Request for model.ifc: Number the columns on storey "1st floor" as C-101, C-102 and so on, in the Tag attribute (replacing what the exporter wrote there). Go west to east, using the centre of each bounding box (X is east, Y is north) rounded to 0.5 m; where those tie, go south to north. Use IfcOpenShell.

First a look at what the model holds.

```python
import ifcopenshell
import ifcopenshell.util.element
import ifcopenshell.util.placement

model = ifcopenshell.open("model.ifc")
print(model.schema)
storey = next(s for s in model.by_type("IfcBuildingStorey") if s.Name == "1st floor")
columns = [e for e in ifcopenshell.util.element.get_decomposition(storey) if e.is_a("IfcColumn")]
for e in sorted(columns, key=lambda e: e.id()):
    origin = ifcopenshell.util.placement.get_local_placement(e.ObjectPlacement)[:3, 3]
    print(e.id(), e.Tag, e.Name, origin.round(2) + 0.0, sep=" | ")
```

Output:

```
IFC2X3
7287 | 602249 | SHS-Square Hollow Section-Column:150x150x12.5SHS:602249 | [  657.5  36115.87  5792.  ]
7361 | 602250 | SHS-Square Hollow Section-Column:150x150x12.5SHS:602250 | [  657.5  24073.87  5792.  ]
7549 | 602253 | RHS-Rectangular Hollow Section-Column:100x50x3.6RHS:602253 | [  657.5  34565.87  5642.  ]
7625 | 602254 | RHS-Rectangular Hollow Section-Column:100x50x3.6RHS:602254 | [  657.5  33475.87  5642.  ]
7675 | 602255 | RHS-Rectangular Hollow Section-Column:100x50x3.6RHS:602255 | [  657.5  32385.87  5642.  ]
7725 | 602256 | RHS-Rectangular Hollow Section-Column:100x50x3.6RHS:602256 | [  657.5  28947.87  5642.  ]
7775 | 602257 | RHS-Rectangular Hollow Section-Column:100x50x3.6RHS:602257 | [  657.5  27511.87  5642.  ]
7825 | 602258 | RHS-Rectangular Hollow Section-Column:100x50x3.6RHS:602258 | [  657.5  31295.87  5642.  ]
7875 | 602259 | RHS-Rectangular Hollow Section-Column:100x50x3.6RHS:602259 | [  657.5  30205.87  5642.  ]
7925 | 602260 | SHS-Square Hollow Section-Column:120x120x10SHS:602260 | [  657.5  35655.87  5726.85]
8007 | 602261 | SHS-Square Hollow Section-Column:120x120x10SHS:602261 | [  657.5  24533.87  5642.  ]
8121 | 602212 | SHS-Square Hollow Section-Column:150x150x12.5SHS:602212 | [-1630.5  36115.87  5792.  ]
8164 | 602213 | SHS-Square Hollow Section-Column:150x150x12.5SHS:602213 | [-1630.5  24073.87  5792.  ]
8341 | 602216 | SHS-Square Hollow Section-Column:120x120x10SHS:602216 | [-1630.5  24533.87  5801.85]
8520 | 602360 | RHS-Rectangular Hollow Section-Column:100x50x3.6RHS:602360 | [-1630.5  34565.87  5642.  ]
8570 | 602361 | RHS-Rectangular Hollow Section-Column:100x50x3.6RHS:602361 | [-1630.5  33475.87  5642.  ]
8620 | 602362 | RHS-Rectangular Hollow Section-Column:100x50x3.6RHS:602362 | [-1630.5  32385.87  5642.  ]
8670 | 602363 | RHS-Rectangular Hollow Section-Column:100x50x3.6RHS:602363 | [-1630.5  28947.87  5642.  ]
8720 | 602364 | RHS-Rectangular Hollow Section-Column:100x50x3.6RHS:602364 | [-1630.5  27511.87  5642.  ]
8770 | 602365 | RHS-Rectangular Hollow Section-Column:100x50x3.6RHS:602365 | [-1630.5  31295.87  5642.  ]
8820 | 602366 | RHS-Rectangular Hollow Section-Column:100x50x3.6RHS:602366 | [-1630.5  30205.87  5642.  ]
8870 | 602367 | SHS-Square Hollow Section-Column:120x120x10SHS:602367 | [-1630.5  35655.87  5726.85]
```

```python
import ifcopenshell
import ifcopenshell.geom
import ifcopenshell.util.element
import ifcopenshell.util.shape

model = ifcopenshell.open("model.ifc")
settings = ifcopenshell.geom.settings()
settings.set("use-world-coords", True)


def centre(element):
    shape = ifcopenshell.geom.create_shape(settings, element)
    return ifcopenshell.util.shape.get_bbox_centroid(shape.geometry)


storey = next(s for s in model.by_type("IfcBuildingStorey") if s.Name == "1st floor")
columns = [e for e in ifcopenshell.util.element.get_decomposition(storey) if e.is_a("IfcColumn")]

# Insertion points can sit at a corner or the storey origin, so sort by the geometry (in metres).
centres = {e: centre(e) for e in columns}
columns.sort(key=lambda e: (round(centres[e][0] / 0.5), centres[e][1]))

for i, e in enumerate(columns, start=1):
    number = f"C-1{i:02d}"
    e.Tag = number
    print(e.id(), number)

model.write("model_updated.ifc")
```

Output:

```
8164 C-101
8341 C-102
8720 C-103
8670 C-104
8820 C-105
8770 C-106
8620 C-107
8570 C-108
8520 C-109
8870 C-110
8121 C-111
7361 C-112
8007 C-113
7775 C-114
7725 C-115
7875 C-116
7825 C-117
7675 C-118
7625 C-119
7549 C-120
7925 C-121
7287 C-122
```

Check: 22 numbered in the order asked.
